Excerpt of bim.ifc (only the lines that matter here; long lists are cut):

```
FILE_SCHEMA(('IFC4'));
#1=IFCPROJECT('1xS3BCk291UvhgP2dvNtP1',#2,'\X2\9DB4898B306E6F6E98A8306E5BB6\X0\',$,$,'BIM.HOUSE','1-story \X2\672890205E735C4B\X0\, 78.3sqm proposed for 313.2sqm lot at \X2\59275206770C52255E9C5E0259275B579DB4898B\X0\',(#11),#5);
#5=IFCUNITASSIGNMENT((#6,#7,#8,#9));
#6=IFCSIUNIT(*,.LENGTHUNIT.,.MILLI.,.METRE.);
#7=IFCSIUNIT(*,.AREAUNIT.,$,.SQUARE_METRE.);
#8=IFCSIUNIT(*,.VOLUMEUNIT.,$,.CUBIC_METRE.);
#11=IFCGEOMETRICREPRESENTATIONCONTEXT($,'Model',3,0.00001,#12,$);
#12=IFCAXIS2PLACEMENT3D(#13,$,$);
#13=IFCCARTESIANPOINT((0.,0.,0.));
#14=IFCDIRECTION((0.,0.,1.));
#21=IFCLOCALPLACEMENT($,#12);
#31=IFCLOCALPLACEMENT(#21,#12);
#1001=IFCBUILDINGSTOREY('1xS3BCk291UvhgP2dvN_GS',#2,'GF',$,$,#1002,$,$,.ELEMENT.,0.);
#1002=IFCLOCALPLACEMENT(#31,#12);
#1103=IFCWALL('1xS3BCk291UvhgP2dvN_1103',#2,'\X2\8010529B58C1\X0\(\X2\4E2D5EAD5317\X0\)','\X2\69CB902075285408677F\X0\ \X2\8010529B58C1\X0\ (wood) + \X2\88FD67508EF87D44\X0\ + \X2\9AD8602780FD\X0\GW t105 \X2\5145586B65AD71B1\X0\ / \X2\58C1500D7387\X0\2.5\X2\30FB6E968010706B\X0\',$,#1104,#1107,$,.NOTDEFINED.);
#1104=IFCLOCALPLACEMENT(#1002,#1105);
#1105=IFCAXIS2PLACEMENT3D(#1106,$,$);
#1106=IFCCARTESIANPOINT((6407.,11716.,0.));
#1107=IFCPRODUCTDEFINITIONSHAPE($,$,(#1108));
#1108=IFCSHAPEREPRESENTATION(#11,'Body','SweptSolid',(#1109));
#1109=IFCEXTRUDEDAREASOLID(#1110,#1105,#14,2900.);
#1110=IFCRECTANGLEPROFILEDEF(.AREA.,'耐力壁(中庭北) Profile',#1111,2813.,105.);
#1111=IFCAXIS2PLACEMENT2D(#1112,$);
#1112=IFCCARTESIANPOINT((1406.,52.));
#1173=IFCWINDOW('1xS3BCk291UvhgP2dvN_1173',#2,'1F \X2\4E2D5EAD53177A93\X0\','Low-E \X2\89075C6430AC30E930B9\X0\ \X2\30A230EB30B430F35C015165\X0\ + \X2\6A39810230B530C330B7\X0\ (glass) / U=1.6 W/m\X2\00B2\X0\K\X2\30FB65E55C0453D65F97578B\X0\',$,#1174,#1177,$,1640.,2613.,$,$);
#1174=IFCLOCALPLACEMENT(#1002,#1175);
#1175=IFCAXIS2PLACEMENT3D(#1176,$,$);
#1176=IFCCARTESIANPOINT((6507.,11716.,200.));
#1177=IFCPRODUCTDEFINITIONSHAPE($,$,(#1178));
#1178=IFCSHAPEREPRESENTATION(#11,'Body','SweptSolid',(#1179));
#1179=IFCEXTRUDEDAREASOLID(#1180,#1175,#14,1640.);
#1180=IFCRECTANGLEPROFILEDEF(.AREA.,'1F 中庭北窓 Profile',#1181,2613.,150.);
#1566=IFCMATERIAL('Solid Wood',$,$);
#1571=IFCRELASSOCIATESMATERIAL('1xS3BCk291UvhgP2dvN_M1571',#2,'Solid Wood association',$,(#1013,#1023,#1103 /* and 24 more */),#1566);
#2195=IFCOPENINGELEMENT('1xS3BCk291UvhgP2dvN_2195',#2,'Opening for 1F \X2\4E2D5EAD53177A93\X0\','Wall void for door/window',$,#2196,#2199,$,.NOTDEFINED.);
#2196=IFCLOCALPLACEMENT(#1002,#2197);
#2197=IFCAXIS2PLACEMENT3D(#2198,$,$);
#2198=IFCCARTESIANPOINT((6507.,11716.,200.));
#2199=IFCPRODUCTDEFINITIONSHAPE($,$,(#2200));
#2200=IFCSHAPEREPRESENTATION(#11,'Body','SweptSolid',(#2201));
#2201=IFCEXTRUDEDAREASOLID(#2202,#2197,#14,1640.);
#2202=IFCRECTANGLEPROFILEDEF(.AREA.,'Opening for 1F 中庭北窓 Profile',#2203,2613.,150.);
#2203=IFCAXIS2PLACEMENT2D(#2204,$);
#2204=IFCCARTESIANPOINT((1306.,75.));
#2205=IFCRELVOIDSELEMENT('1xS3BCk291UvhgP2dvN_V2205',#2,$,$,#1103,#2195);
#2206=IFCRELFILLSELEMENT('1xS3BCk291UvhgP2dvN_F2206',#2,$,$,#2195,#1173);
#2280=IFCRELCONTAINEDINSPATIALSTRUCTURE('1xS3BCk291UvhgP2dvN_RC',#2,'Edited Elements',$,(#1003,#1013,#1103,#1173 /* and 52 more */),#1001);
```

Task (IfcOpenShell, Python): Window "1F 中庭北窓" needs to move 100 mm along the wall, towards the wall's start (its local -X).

```python
import ifcopenshell
import ifcopenshell.api.geometry
import ifcopenshell.util.placement
import ifcopenshell.util.unit

model = ifcopenshell.open("bim.ifc")
unit_scale = ifcopenshell.util.unit.calculate_unit_scale(model)

window = model.by_guid("1xS3BCk291UvhgP2dvN_1173")
opening = window.FillsVoids[0].RelatingOpeningElement
wall = opening.VoidsElements[0].RelatingBuildingElement

wall_matrix = ifcopenshell.util.placement.get_local_placement(wall.ObjectPlacement)
shift = wall_matrix[:3, 0] * -0.1 / unit_scale
before = ifcopenshell.util.placement.get_local_placement(window.ObjectPlacement)[:3, 3].copy()

# The window is not placed relative to its opening, so move both.
for product in (opening, window):
    matrix = ifcopenshell.util.placement.get_local_placement(product.ObjectPlacement)
    matrix[:3, 3] += shift
    ifcopenshell.api.geometry.edit_object_placement(model, product=product, matrix=matrix, is_si=False)

after = ifcopenshell.util.placement.get_local_placement(window.ObjectPlacement)[:3, 3]
print("window moved by", (after - before).round(3) + 0.0)

model.write("bim_edited.ifc")
```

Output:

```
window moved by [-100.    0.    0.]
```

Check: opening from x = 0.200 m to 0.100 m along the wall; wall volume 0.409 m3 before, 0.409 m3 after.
